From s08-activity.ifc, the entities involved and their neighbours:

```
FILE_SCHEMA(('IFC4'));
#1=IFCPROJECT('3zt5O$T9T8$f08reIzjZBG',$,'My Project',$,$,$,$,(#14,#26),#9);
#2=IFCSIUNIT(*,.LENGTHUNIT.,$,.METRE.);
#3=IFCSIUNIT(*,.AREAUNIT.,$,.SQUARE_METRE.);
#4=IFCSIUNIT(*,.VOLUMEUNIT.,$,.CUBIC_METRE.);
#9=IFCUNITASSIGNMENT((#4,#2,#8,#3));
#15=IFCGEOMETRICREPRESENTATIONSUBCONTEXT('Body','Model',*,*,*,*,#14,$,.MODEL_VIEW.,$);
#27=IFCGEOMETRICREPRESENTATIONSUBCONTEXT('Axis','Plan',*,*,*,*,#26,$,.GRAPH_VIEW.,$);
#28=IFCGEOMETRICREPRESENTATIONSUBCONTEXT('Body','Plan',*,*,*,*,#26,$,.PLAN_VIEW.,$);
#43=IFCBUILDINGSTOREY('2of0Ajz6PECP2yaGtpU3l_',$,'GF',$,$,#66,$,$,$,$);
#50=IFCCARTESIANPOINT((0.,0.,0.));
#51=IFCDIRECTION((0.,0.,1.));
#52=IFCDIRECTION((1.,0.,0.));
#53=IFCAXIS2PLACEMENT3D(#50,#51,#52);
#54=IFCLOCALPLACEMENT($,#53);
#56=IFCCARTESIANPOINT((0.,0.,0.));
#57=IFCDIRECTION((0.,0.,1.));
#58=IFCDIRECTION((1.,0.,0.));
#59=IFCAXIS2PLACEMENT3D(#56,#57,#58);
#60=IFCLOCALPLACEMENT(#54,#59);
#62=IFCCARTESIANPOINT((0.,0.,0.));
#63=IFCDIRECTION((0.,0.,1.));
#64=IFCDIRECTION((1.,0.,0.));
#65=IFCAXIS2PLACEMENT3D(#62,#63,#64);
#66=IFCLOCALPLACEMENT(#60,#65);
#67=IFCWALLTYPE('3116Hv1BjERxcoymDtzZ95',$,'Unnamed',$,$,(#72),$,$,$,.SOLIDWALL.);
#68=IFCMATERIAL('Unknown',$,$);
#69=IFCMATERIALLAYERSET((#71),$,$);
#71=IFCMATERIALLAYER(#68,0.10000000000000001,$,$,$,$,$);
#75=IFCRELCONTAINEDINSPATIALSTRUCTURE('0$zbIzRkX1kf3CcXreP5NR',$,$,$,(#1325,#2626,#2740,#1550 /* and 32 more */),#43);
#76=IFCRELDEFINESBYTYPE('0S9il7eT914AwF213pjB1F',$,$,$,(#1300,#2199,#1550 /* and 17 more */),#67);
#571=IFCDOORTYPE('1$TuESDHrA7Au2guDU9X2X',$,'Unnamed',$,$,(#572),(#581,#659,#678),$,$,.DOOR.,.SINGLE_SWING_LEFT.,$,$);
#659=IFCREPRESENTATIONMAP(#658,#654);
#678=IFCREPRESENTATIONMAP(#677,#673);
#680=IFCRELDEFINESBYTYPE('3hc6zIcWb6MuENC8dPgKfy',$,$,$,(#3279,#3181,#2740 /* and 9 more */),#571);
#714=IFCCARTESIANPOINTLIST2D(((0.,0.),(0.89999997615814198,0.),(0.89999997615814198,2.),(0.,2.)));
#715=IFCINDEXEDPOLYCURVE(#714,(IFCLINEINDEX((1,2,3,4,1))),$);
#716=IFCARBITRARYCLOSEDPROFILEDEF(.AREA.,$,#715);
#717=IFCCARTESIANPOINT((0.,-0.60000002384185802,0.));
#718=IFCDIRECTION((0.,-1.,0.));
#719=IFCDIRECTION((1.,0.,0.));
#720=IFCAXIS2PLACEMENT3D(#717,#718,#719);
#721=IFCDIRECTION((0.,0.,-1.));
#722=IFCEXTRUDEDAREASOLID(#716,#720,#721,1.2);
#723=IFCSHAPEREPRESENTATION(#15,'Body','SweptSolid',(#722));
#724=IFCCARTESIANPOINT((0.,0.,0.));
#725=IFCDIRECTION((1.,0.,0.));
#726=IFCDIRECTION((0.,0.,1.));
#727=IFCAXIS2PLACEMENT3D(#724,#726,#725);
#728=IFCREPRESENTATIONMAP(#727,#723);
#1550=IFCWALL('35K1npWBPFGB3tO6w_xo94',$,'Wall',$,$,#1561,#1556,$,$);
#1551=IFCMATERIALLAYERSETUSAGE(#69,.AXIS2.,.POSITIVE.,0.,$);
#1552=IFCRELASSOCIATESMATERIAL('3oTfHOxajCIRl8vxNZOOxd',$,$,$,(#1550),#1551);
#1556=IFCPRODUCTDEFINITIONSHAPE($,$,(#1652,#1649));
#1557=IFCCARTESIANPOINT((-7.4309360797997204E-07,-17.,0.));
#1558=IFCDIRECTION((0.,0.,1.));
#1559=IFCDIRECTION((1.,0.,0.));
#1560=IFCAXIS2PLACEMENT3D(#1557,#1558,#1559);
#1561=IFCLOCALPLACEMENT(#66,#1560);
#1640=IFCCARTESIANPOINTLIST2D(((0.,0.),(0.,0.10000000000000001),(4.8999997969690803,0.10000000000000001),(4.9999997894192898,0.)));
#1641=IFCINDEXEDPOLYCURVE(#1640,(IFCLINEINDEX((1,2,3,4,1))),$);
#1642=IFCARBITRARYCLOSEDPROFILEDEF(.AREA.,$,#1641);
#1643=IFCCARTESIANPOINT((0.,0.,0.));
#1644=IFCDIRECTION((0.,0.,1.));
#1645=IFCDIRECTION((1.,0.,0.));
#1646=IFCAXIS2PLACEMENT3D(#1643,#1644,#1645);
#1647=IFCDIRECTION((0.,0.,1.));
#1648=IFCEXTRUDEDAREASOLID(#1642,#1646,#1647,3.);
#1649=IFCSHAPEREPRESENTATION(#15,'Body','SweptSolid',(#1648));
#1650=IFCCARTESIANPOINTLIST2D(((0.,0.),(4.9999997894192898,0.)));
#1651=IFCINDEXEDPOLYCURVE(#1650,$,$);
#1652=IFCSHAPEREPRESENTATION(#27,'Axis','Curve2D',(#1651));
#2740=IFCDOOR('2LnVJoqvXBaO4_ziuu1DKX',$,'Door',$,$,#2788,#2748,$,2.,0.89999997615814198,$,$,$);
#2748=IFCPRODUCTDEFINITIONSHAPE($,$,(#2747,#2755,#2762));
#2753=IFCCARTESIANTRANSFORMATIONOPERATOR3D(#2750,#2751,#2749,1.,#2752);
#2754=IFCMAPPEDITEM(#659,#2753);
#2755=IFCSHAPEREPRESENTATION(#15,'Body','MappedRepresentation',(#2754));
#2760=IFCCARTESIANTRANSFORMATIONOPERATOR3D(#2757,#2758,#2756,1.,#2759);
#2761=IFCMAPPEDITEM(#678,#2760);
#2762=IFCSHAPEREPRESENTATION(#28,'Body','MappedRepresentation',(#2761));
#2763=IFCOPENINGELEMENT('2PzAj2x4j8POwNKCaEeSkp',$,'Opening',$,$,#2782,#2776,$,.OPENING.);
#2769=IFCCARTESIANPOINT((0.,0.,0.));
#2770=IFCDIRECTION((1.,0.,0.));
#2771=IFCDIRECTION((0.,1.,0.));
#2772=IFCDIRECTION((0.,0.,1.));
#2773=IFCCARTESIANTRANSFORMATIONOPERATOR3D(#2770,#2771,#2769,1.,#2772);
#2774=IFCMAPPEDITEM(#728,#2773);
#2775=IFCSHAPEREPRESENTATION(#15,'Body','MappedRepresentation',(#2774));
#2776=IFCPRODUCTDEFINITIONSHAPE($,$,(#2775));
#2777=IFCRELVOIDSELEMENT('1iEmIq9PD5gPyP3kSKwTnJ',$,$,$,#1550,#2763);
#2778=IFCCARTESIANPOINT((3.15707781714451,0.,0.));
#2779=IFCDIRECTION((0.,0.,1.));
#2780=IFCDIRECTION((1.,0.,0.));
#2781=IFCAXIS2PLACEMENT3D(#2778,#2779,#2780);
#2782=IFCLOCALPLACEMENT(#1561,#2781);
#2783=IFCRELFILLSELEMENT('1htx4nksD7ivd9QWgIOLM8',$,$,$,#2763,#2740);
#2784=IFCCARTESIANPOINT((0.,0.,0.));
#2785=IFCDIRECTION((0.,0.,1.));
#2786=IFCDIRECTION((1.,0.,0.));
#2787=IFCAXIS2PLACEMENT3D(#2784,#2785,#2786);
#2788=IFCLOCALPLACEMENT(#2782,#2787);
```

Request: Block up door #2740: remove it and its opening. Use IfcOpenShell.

```python
import ifcopenshell
import ifcopenshell.api.feature
import ifcopenshell.api.root
import ifcopenshell.geom
import ifcopenshell.util.shape

model = ifcopenshell.open("s08-activity.ifc")
settings = ifcopenshell.geom.settings()


def volume(element):
    """Net volume in cubic metres, openings subtracted."""
    shape = ifcopenshell.geom.create_shape(settings, element)
    return ifcopenshell.util.shape.get_volume(shape.geometry)


door = model.by_guid("2LnVJoqvXBaO4_ziuu1DKX")
opening = door.FillsVoids[0].RelatingOpeningElement
wall = opening.VoidsElements[0].RelatingBuildingElement
before = volume(wall)

ifcopenshell.api.root.remove_product(model, product=door)
ifcopenshell.api.feature.remove_feature(model, feature=opening)

after = volume(wall)

print(f"wall volume {before:.3f} -> {after:.3f} m3")

model.write("s08-activity_edited.ifc")
```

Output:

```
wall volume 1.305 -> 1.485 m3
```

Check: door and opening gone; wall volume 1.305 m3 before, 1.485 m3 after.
